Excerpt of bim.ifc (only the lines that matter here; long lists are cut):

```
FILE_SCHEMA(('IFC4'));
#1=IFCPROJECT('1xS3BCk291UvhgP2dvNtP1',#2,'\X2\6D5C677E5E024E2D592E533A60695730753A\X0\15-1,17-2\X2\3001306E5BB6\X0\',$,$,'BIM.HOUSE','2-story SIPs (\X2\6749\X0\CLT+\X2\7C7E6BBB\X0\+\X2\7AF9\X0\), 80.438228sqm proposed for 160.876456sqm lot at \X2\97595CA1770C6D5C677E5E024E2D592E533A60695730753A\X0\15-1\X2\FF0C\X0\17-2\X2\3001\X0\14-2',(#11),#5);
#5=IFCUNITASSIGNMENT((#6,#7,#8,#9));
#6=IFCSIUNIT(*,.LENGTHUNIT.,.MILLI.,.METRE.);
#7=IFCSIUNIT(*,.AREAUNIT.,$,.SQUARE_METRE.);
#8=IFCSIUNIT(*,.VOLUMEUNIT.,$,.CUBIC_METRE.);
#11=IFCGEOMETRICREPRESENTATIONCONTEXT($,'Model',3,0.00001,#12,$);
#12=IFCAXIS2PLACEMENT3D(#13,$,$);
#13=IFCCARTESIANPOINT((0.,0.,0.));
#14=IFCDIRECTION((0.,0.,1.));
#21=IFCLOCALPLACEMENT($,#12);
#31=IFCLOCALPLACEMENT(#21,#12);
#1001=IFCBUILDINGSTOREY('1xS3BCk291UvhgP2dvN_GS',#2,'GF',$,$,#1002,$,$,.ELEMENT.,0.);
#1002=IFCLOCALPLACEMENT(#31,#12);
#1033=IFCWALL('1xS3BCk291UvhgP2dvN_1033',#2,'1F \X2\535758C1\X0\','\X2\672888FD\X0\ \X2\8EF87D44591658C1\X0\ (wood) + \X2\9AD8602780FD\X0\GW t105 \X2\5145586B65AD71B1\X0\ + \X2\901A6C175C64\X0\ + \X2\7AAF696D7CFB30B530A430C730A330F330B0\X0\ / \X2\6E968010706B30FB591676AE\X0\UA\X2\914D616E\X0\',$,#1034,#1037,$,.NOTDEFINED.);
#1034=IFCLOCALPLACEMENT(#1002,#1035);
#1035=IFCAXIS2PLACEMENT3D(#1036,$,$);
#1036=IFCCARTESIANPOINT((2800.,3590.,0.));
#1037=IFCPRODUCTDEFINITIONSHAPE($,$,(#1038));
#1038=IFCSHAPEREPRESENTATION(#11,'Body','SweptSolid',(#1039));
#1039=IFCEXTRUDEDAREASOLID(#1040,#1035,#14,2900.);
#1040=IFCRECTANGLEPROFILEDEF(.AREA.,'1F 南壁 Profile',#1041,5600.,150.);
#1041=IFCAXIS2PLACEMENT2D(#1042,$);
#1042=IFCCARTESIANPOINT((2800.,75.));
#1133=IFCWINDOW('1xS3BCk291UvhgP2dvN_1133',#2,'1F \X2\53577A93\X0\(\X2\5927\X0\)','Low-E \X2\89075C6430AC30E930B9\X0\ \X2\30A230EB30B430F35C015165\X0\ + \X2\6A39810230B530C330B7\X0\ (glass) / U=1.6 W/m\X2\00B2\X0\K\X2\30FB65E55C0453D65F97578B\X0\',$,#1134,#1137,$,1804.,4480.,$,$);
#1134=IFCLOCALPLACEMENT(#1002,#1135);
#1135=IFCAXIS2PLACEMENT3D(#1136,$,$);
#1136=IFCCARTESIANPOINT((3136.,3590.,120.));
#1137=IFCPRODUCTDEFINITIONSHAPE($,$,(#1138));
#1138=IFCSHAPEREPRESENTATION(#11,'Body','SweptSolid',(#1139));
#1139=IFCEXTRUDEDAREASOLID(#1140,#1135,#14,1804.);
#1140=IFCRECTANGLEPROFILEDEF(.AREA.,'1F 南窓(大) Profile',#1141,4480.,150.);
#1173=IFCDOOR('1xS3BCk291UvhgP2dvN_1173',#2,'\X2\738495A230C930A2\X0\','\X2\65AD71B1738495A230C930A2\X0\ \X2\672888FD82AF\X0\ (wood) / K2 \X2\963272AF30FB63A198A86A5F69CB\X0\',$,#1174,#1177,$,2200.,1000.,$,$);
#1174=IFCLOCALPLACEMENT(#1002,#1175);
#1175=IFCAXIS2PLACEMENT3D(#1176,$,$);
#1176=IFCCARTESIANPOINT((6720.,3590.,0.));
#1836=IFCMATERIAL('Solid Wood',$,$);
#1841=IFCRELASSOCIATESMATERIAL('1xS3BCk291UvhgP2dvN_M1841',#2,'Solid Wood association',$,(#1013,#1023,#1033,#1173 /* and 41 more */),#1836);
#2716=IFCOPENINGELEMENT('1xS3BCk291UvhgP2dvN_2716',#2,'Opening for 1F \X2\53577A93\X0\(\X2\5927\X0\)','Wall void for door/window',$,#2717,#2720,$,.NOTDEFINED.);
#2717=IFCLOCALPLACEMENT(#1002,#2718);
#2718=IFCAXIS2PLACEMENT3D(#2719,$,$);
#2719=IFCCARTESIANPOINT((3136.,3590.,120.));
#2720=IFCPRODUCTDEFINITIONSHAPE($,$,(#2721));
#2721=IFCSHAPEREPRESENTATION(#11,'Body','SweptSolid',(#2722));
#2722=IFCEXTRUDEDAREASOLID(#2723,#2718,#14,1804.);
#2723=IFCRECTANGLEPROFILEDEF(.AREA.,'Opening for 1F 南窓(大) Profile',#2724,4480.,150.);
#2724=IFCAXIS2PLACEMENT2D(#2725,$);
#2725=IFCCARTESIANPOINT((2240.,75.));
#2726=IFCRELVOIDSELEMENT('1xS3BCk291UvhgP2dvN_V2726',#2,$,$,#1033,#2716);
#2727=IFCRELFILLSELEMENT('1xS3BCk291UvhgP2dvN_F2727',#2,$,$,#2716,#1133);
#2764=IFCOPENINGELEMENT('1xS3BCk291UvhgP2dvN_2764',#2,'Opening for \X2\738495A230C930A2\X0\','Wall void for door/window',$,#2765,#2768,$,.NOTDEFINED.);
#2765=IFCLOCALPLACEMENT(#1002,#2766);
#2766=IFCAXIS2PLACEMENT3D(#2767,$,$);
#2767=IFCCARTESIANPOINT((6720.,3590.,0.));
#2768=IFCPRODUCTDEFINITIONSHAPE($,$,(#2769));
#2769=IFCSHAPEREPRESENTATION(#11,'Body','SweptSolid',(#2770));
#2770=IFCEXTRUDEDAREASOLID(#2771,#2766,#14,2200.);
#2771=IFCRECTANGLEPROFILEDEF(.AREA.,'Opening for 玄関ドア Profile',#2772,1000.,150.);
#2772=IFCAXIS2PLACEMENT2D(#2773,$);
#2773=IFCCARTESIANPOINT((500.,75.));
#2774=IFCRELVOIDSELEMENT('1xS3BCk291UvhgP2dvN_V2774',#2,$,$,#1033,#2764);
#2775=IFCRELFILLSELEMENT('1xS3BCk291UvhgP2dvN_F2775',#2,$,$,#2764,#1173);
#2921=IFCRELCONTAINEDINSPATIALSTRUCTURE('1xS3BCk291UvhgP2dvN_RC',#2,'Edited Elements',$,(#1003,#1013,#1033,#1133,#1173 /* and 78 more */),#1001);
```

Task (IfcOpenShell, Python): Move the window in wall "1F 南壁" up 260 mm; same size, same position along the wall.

```python
import numpy as np
import ifcopenshell
import ifcopenshell.api.geometry
import ifcopenshell.util.placement
import ifcopenshell.util.unit

model = ifcopenshell.open("bim.ifc")
unit_scale = ifcopenshell.util.unit.calculate_unit_scale(model)

window = model.by_id(1133)
opening = window.FillsVoids[0].RelatingOpeningElement
dz = 0.26 / unit_scale

shift = np.array([0.0, 0.0, dz])
# The window is not placed relative to its opening, so move both.
for product in (opening, window):
    matrix = ifcopenshell.util.placement.get_local_placement(product.ObjectPlacement)
    matrix[:3, 3] += shift
    ifcopenshell.api.geometry.edit_object_placement(model, product=product, matrix=matrix, is_si=False)

print(f"moved by {dz * unit_scale:+.3f} m")

model.write("bim_v2.ifc")
```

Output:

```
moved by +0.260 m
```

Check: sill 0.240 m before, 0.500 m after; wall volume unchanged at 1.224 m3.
